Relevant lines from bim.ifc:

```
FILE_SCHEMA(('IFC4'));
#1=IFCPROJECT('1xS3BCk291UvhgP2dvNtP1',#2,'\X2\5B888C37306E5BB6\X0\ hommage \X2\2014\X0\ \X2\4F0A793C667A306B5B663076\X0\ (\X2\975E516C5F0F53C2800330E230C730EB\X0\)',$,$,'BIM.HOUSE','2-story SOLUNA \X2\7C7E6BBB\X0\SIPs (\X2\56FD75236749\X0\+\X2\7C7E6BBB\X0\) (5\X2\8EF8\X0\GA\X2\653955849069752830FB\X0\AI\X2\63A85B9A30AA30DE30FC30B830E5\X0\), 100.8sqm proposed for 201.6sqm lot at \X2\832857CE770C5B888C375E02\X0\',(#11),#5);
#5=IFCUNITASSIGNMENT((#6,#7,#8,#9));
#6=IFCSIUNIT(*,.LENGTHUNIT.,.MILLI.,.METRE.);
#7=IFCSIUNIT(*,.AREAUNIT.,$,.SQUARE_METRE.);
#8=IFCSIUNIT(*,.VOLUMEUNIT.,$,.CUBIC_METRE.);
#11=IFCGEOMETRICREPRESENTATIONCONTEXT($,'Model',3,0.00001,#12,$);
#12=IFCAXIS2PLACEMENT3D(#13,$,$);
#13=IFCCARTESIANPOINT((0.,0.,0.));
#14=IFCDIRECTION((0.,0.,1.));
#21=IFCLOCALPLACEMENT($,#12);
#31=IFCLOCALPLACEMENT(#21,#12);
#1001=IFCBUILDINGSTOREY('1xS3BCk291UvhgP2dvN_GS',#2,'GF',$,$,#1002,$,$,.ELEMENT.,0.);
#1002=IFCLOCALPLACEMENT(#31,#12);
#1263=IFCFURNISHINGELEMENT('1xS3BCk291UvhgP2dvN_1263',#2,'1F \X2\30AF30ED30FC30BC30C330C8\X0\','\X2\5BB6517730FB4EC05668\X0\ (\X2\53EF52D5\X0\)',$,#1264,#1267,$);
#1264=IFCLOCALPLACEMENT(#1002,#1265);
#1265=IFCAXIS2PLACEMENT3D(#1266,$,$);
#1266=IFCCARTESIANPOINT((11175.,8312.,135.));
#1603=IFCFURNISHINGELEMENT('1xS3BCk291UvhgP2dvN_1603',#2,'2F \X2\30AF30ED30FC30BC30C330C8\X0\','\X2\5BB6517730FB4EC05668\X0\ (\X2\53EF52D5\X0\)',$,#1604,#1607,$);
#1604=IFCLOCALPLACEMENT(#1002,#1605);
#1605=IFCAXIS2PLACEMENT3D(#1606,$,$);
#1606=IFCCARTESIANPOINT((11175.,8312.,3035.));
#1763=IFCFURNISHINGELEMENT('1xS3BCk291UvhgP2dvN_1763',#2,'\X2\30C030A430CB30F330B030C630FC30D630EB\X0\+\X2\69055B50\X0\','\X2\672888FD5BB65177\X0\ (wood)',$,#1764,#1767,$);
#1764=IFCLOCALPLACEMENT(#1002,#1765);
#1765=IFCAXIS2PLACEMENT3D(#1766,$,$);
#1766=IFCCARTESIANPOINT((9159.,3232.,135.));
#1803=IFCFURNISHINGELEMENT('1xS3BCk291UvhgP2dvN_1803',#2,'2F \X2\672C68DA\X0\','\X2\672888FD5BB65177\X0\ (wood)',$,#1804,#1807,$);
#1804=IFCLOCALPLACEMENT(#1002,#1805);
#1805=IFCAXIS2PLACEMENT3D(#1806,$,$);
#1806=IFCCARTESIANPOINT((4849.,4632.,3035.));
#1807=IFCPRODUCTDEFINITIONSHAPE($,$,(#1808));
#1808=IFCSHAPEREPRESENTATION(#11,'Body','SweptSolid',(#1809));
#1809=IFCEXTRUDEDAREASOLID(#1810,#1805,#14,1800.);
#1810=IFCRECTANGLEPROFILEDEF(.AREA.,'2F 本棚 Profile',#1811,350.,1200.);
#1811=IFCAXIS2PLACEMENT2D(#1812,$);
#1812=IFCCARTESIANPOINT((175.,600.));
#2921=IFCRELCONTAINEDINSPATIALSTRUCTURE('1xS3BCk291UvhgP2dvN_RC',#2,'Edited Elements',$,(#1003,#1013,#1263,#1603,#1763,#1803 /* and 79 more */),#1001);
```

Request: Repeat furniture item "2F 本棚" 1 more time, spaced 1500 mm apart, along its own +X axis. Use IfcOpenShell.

```python
import ifcopenshell
import ifcopenshell.api.geometry
import ifcopenshell.api.root
import ifcopenshell.util.element
import ifcopenshell.util.placement
import ifcopenshell.util.unit

model = ifcopenshell.open("bim.ifc")
unit_scale = ifcopenshell.util.unit.calculate_unit_scale(model)


def reuse_history(source, copy):
    """copy_class also copies each property set's owner history, people and application; keep the originals."""
    for rel in copy.IsDefinedBy:
        if rel.is_a("IfcRelDefinesByProperties") and (history := rel.RelatingPropertyDefinition.OwnerHistory):
            rel.RelatingPropertyDefinition.OwnerHistory = source.OwnerHistory
            ifcopenshell.util.element.remove_deep2(model, history)


source = model.by_guid("1xS3BCk291UvhgP2dvN_1803")
base = ifcopenshell.util.placement.get_local_placement(source.ObjectPlacement)
step = base[:3, 0] * 1.5 / unit_scale

for i in range(1, 2):
    copy = ifcopenshell.api.root.copy_class(model, product=source)
    copy.Representation = ifcopenshell.util.element.copy_deep(
        model, source.Representation, exclude=["IfcGeometricRepresentationContext", "IfcRepresentationMap"]
    )
    reuse_history(source, copy)
    matrix = base.copy()
    matrix[:3, 3] += i * step
    print("added at", matrix[:3, 3].round(3) + 0.0)
    ifcopenshell.api.geometry.edit_object_placement(model, product=copy, matrix=matrix, is_si=False)

model.write("bim-out.ifc")
```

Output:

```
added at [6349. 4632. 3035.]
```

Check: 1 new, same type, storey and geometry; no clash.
